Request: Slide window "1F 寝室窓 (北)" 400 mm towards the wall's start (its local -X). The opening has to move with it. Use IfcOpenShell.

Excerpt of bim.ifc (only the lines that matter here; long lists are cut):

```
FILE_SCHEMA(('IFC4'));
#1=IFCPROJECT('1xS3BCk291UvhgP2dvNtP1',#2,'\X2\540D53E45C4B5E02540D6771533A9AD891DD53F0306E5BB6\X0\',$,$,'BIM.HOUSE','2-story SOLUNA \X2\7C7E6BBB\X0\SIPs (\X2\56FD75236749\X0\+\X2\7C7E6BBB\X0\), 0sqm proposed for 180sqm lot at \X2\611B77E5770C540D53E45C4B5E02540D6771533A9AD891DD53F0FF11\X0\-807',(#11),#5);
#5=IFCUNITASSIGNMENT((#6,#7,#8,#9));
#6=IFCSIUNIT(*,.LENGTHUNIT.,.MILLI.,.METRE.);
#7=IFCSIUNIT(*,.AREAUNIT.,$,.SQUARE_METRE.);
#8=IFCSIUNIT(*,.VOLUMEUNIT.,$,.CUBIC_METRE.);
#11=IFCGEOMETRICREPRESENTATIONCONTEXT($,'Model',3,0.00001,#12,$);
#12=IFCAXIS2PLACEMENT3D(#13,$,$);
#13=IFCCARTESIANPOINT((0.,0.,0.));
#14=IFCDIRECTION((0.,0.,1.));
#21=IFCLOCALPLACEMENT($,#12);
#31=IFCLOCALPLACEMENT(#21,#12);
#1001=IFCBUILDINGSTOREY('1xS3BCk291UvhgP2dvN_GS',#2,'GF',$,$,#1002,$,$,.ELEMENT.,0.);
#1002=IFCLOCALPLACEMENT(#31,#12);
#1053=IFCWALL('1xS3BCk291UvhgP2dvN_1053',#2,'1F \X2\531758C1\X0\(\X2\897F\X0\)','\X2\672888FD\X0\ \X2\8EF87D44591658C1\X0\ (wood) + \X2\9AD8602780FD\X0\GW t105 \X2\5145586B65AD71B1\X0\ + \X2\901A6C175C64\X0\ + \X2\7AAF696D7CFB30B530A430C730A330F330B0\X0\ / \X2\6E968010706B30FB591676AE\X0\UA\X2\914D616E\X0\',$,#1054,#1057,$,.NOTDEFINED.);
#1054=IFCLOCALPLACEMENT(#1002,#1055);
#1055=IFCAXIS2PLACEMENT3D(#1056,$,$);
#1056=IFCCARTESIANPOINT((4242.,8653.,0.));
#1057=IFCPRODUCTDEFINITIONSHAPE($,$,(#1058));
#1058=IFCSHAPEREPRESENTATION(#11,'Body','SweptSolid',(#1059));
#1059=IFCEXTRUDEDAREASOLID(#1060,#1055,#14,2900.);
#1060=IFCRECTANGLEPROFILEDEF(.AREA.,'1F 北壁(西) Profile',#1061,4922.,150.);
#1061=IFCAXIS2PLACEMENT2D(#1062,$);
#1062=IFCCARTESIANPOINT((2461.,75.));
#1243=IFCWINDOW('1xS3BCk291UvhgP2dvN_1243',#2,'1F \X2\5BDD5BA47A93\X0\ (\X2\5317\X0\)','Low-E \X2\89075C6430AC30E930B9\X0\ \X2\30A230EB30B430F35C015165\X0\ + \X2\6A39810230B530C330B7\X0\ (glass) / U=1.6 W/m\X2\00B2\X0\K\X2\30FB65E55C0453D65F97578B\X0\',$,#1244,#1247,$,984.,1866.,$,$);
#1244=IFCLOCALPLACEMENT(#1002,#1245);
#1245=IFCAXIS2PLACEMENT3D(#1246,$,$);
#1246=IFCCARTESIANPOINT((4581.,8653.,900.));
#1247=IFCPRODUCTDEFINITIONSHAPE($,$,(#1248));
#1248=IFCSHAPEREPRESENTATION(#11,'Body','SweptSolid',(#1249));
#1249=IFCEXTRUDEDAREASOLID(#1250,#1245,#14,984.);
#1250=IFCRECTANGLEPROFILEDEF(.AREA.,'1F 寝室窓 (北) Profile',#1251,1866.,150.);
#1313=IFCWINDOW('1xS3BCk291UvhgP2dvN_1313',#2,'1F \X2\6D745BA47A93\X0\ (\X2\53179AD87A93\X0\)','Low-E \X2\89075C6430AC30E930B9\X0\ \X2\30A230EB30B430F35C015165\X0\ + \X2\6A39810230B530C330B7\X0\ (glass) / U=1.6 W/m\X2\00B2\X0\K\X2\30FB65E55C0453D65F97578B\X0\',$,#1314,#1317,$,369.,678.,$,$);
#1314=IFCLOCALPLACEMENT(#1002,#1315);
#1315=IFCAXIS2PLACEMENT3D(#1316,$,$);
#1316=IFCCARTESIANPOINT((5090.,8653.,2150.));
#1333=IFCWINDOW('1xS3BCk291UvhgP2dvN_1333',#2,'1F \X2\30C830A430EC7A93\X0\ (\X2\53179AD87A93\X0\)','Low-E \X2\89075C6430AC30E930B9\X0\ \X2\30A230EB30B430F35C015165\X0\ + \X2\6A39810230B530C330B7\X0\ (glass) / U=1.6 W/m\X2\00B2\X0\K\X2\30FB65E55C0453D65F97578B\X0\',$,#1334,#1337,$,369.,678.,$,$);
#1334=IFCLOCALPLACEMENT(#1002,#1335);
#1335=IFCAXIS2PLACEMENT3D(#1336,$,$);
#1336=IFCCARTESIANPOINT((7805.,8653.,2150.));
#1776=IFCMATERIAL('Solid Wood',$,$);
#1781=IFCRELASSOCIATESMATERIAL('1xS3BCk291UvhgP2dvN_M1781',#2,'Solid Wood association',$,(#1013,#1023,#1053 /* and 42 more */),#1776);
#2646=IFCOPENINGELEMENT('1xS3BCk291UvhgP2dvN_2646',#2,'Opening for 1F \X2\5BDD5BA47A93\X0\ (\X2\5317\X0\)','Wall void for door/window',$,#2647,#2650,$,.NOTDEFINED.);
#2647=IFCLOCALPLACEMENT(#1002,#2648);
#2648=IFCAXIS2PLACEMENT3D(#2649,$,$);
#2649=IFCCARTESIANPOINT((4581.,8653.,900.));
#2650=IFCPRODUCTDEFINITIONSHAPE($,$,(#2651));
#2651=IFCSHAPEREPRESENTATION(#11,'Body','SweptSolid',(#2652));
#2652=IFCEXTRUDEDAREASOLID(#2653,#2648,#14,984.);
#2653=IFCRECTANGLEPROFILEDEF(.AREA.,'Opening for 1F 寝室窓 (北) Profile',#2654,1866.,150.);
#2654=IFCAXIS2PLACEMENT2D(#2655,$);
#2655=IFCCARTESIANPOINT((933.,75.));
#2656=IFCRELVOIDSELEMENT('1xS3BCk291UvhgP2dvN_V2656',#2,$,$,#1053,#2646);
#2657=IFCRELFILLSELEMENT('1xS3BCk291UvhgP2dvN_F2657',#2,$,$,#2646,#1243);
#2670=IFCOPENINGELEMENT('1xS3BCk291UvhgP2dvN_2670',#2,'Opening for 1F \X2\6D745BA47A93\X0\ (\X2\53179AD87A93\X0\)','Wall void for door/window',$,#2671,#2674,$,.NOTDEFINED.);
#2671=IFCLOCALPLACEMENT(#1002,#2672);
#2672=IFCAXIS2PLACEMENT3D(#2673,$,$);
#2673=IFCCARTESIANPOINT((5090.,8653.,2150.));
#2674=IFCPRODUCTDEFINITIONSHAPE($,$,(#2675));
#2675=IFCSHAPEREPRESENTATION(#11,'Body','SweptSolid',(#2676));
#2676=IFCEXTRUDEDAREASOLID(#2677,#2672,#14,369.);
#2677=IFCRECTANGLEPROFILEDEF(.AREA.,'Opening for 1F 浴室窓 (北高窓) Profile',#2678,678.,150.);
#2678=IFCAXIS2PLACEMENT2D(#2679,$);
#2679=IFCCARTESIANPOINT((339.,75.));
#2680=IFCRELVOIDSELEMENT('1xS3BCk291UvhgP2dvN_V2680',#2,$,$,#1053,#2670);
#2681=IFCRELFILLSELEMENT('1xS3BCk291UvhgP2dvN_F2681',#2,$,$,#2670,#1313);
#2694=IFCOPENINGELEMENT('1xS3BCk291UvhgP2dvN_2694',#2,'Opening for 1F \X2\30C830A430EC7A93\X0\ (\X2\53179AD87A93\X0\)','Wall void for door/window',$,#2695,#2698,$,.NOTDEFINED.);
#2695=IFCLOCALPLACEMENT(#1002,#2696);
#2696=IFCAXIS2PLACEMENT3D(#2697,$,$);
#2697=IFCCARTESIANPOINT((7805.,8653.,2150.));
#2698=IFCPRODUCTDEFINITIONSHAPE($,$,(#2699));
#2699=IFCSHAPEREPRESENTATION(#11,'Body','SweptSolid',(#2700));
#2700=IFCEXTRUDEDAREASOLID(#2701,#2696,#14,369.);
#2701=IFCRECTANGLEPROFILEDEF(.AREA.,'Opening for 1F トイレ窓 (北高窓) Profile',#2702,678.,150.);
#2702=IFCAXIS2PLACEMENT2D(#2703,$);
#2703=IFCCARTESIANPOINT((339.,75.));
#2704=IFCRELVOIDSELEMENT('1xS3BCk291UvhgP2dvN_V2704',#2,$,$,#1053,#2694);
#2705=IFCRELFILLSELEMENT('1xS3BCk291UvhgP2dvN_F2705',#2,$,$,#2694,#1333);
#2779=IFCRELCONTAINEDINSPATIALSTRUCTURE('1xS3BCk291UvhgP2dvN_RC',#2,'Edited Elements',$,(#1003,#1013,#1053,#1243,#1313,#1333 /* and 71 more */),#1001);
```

```python
import ifcopenshell
import ifcopenshell.api.geometry
import ifcopenshell.util.placement

model = ifcopenshell.open("bim.ifc")

window = model.by_guid("1xS3BCk291UvhgP2dvN_1243")
opening = window.FillsVoids[0].RelatingOpeningElement
wall = opening.VoidsElements[0].RelatingBuildingElement

wall_matrix = ifcopenshell.util.placement.get_local_placement(wall.ObjectPlacement)
shift = wall_matrix[:3, 0] * -400.0
before = ifcopenshell.util.placement.get_local_placement(window.ObjectPlacement)[:3, 3].copy()

# The window is not placed relative to its opening, so move both.
for product in (opening, window):
    matrix = ifcopenshell.util.placement.get_local_placement(product.ObjectPlacement)
    matrix[:3, 3] += shift
    ifcopenshell.api.geometry.edit_object_placement(model, product=product, matrix=matrix, is_si=False)

after = ifcopenshell.util.placement.get_local_placement(window.ObjectPlacement)[:3, 3]
print("window moved by", (after - before).round(3) + 0.0)

model.write("bim_v2.ifc")
```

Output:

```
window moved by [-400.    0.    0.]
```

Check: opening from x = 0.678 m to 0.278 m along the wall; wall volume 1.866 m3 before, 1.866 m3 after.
